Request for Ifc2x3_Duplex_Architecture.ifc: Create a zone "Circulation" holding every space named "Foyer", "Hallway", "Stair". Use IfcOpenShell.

First a look at what the model holds.

```python
import ifcopenshell

model = ifcopenshell.open("Ifc2x3_Duplex_Architecture.ifc")
print(model.schema)
seen = {}
for space in model.by_type("IfcSpace"):
    seen[space.LongName] = seen.get(space.LongName, 0) + 1
for name, count in sorted(seen.items(), key=str):
    print(count, "x", name)
print("zones:", [z.Name for z in model.by_type("IfcZone")][:20])
```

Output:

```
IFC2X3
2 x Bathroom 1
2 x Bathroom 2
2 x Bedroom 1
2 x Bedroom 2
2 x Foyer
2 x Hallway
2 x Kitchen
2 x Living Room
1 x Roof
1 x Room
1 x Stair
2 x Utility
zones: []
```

```python
import ifcopenshell
import ifcopenshell.api.group
import ifcopenshell.api.root

model = ifcopenshell.open("Ifc2x3_Duplex_Architecture.ifc")

names = {"Foyer", "Hallway", "Stair"}
spaces = [s for s in model.by_type("IfcSpace") if s.LongName in names]

zone = ifcopenshell.api.root.create_entity(model, ifc_class="IfcZone", name="Circulation")
ifcopenshell.api.group.assign_group(model, products=spaces, group=zone)
print(len(spaces), "spaces in", zone.Name)

model.write("Ifc2x3_Duplex_Architecture_rev.ifc")
```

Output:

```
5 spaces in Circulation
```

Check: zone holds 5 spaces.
